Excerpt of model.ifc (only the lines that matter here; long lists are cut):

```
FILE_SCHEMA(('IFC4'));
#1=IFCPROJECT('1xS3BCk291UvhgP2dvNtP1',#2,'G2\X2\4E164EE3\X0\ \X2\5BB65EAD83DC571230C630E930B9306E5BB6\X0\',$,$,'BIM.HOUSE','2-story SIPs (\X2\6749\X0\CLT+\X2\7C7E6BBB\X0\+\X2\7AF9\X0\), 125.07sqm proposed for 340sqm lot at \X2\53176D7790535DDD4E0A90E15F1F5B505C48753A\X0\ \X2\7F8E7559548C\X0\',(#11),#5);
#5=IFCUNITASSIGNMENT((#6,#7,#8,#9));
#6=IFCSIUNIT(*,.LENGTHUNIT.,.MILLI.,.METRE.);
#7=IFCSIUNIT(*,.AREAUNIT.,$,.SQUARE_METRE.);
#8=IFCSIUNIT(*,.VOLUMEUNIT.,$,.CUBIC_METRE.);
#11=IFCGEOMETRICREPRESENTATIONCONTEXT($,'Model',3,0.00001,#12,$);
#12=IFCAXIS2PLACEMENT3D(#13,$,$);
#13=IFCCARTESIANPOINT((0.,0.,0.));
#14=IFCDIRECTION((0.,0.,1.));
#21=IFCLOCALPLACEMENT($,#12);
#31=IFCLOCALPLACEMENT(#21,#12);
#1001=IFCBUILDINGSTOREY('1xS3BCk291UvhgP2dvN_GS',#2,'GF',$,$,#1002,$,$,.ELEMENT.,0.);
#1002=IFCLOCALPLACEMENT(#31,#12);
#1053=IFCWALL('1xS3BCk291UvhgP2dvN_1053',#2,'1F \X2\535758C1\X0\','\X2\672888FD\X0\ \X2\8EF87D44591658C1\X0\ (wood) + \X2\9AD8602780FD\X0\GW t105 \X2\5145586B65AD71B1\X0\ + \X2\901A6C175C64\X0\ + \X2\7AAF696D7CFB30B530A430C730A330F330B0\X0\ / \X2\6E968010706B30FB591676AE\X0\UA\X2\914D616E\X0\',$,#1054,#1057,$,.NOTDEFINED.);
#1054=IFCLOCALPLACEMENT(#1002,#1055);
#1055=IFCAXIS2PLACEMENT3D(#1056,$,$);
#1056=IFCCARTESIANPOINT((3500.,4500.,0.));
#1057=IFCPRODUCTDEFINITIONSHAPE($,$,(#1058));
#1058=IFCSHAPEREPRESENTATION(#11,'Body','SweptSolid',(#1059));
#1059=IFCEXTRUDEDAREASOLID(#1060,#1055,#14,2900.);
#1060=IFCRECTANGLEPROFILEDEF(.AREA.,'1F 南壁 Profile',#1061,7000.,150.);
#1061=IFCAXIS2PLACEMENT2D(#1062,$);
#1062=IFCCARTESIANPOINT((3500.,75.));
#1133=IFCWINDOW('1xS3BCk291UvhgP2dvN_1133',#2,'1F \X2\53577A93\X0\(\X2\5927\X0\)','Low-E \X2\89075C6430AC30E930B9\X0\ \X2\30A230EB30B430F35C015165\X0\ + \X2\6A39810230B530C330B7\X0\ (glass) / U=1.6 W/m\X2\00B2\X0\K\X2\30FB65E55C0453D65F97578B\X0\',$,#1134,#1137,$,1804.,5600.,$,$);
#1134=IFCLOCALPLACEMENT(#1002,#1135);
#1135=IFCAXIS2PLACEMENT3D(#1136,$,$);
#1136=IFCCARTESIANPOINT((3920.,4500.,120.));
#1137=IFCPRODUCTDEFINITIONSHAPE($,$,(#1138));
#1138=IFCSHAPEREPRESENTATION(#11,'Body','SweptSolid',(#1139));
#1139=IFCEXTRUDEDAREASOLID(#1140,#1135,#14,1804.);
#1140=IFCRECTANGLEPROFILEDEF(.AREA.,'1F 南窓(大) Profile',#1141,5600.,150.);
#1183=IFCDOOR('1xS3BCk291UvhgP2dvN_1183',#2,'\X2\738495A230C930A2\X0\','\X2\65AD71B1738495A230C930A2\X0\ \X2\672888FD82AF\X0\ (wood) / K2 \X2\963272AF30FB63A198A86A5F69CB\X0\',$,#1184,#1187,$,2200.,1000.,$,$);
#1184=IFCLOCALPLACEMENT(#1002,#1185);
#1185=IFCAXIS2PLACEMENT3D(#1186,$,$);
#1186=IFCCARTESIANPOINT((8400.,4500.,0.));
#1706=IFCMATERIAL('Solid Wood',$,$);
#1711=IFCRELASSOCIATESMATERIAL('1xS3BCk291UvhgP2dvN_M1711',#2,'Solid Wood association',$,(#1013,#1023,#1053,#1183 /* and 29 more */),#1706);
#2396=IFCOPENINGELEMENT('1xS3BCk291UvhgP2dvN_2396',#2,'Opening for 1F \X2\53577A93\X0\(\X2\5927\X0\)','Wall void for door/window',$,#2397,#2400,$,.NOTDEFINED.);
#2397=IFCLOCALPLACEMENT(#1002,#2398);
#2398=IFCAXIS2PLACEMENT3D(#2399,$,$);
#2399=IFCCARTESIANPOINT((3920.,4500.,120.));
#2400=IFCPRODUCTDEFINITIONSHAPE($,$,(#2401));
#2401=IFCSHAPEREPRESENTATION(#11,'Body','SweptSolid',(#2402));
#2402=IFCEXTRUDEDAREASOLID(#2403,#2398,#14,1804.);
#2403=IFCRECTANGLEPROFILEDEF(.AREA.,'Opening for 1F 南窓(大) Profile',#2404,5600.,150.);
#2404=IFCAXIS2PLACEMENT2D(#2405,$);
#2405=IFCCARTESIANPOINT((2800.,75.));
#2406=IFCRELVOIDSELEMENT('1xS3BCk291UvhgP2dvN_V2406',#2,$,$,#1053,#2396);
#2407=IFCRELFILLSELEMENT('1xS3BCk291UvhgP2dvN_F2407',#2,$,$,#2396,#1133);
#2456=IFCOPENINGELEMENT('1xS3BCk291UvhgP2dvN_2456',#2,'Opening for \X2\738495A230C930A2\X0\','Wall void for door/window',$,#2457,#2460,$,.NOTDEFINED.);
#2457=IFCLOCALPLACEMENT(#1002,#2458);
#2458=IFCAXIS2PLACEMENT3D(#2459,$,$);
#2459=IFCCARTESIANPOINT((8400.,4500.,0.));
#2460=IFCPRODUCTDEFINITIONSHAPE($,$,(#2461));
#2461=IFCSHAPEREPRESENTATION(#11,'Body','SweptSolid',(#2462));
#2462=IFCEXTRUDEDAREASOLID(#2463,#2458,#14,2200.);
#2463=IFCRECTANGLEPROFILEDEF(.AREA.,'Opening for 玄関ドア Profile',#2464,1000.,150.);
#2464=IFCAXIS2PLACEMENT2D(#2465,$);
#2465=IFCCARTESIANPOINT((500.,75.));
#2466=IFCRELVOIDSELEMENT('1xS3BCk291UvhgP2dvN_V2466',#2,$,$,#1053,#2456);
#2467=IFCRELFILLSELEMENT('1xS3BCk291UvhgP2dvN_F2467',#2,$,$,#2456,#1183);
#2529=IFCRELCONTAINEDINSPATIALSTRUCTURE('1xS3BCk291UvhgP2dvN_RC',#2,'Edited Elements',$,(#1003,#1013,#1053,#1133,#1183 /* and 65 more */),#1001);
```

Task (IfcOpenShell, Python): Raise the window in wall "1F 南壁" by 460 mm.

```python
import numpy as np
import ifcopenshell
import ifcopenshell.api.geometry
import ifcopenshell.util.placement
import ifcopenshell.util.unit

model = ifcopenshell.open("model.ifc")
unit_scale = ifcopenshell.util.unit.calculate_unit_scale(model)

window = model.by_guid("1xS3BCk291UvhgP2dvN_1133")
opening = window.FillsVoids[0].RelatingOpeningElement
dz = 460.0

shift = np.array([0.0, 0.0, dz])
# The window is not placed relative to its opening, so move both.
for product in (opening, window):
    matrix = ifcopenshell.util.placement.get_local_placement(product.ObjectPlacement)
    matrix[:3, 3] += shift
    ifcopenshell.api.geometry.edit_object_placement(model, product=product, matrix=matrix, is_si=False)

print(f"moved by {dz * unit_scale:+.3f} m")

model.write("model_v2.ifc")
```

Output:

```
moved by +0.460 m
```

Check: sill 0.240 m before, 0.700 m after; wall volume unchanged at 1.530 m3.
